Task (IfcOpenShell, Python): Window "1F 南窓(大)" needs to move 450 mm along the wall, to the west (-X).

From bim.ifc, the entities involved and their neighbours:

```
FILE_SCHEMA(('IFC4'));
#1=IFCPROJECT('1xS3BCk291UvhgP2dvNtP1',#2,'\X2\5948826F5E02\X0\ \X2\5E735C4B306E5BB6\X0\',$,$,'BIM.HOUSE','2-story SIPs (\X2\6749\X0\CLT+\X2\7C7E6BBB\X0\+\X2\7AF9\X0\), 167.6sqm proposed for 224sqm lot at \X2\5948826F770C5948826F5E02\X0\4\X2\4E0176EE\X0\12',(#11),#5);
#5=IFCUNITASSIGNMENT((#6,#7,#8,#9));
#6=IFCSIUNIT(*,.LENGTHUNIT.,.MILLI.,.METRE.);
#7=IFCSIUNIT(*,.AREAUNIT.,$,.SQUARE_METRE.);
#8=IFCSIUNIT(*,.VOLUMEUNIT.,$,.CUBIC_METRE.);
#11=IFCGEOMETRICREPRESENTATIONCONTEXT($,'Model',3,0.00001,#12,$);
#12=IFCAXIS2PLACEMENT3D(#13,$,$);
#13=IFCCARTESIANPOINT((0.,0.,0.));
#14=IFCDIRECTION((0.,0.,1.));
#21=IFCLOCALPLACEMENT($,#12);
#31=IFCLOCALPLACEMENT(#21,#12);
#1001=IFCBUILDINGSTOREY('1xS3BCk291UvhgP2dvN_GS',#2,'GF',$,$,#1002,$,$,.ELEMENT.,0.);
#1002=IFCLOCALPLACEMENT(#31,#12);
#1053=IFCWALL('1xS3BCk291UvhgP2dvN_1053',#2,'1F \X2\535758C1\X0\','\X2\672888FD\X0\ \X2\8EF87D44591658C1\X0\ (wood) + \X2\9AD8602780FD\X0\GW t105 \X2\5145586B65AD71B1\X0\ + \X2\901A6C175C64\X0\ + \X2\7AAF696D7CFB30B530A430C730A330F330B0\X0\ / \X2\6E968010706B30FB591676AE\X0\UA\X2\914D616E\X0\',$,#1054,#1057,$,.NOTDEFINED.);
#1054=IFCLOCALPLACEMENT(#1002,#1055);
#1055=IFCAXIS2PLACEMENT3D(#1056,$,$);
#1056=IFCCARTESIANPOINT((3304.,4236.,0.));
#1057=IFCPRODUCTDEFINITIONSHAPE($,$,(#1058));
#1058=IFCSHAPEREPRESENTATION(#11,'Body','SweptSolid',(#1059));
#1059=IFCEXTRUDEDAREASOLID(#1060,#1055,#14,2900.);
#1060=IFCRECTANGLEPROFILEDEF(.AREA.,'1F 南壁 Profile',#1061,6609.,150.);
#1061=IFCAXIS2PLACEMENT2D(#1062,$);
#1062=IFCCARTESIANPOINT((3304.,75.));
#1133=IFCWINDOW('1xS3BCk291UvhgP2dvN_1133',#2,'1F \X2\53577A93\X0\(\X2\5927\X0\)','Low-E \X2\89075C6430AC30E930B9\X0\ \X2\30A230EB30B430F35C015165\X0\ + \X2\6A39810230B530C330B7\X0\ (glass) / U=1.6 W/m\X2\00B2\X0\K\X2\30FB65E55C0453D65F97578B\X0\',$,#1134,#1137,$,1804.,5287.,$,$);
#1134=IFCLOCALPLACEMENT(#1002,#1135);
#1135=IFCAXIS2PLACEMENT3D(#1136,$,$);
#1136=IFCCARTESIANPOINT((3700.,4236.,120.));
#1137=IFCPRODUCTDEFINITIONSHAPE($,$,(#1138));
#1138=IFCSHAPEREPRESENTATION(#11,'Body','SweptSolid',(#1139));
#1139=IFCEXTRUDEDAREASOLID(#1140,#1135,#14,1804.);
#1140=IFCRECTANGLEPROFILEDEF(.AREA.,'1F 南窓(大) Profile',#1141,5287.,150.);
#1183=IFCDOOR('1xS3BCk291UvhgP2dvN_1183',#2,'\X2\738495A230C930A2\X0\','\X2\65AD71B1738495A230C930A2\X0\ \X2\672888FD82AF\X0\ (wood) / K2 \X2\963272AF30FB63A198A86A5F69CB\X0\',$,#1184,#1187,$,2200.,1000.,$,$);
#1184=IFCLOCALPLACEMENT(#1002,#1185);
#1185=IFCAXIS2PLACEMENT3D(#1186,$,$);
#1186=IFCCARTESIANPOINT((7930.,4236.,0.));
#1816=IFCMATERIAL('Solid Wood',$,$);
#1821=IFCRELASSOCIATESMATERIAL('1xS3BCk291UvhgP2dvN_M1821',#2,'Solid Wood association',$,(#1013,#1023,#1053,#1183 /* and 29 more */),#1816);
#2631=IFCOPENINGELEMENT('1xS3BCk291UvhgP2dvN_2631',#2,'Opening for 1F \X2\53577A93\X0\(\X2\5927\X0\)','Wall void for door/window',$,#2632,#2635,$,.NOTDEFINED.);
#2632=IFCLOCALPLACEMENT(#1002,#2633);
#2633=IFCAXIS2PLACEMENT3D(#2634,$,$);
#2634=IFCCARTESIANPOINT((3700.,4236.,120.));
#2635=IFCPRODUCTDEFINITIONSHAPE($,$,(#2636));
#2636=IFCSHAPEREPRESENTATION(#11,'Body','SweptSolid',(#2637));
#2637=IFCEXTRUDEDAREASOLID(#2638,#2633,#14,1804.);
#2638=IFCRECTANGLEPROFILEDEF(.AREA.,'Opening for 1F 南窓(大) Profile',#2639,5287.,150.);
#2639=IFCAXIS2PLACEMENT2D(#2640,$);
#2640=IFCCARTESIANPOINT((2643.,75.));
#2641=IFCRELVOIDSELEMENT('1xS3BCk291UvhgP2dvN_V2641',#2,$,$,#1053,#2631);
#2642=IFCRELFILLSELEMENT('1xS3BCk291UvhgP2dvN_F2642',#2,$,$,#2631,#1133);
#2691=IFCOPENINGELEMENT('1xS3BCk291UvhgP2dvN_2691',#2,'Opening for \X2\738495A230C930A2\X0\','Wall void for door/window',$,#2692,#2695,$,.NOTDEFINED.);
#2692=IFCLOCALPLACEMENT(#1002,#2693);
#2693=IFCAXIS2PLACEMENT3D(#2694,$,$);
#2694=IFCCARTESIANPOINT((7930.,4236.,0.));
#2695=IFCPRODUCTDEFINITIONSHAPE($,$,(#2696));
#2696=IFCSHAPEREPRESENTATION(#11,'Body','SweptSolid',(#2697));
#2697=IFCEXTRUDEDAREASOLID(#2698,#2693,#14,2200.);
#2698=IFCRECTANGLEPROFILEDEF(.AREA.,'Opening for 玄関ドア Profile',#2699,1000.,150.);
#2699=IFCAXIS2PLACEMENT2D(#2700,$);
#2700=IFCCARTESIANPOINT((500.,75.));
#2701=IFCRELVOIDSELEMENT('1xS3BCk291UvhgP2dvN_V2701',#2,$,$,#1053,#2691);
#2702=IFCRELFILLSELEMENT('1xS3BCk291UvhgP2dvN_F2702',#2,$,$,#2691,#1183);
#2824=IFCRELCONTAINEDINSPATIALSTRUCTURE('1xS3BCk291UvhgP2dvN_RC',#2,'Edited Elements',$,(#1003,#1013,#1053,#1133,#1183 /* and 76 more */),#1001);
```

```python
import ifcopenshell
import ifcopenshell.api.geometry
import ifcopenshell.util.placement
import ifcopenshell.util.unit

model = ifcopenshell.open("bim.ifc")
unit_scale = ifcopenshell.util.unit.calculate_unit_scale(model)

window = model.by_id(1133)
opening = window.FillsVoids[0].RelatingOpeningElement
wall = opening.VoidsElements[0].RelatingBuildingElement

wall_matrix = ifcopenshell.util.placement.get_local_placement(wall.ObjectPlacement)
shift = wall_matrix[:3, 0] * -0.45 / unit_scale
before = ifcopenshell.util.placement.get_local_placement(window.ObjectPlacement)[:3, 3].copy()

# The window is not placed relative to its opening, so move both.
for product in (opening, window):
    matrix = ifcopenshell.util.placement.get_local_placement(product.ObjectPlacement)
    matrix[:3, 3] += shift
    ifcopenshell.api.geometry.edit_object_placement(model, product=product, matrix=matrix, is_si=False)

after = ifcopenshell.util.placement.get_local_placement(window.ObjectPlacement)[:3, 3]
print("window moved by", (after - before).round(3) + 0.0)

model.write("bim_v2.ifc")
```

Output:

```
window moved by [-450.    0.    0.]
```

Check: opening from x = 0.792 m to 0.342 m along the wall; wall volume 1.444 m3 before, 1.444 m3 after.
